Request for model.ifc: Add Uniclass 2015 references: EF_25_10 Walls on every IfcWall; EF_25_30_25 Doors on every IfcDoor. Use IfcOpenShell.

First a look at what the model holds.

```python
import ifcopenshell

model = ifcopenshell.open("model.ifc")
print(model.schema)
print("classifications:", [c.Name for c in model.by_type("IfcClassification")])
for ifc_class in ("IfcDoor", "IfcRoof", "IfcStair", "IfcWall", "IfcWindow"):
    print(ifc_class, len(model.by_type(ifc_class)))
```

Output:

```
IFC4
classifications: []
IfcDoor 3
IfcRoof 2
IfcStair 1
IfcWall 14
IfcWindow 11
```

```python
import ifcopenshell
import ifcopenshell.api.classification

model = ifcopenshell.open("model.ifc")

system = ifcopenshell.api.classification.add_classification(model, classification="Uniclass 2015")

codes = {
    "IfcWall": ("EF_25_10", "Walls"),
    "IfcDoor": ("EF_25_30_25", "Doors"),
}
for ifc_class, (code, name) in codes.items():
    products = model.by_type(ifc_class)
    ifcopenshell.api.classification.add_reference(
        model, products=products, classification=system, identification=code, name=name
    )
    print(code, len(products))

model.write("model-out.ifc")
```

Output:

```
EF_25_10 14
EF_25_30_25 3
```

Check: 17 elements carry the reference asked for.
